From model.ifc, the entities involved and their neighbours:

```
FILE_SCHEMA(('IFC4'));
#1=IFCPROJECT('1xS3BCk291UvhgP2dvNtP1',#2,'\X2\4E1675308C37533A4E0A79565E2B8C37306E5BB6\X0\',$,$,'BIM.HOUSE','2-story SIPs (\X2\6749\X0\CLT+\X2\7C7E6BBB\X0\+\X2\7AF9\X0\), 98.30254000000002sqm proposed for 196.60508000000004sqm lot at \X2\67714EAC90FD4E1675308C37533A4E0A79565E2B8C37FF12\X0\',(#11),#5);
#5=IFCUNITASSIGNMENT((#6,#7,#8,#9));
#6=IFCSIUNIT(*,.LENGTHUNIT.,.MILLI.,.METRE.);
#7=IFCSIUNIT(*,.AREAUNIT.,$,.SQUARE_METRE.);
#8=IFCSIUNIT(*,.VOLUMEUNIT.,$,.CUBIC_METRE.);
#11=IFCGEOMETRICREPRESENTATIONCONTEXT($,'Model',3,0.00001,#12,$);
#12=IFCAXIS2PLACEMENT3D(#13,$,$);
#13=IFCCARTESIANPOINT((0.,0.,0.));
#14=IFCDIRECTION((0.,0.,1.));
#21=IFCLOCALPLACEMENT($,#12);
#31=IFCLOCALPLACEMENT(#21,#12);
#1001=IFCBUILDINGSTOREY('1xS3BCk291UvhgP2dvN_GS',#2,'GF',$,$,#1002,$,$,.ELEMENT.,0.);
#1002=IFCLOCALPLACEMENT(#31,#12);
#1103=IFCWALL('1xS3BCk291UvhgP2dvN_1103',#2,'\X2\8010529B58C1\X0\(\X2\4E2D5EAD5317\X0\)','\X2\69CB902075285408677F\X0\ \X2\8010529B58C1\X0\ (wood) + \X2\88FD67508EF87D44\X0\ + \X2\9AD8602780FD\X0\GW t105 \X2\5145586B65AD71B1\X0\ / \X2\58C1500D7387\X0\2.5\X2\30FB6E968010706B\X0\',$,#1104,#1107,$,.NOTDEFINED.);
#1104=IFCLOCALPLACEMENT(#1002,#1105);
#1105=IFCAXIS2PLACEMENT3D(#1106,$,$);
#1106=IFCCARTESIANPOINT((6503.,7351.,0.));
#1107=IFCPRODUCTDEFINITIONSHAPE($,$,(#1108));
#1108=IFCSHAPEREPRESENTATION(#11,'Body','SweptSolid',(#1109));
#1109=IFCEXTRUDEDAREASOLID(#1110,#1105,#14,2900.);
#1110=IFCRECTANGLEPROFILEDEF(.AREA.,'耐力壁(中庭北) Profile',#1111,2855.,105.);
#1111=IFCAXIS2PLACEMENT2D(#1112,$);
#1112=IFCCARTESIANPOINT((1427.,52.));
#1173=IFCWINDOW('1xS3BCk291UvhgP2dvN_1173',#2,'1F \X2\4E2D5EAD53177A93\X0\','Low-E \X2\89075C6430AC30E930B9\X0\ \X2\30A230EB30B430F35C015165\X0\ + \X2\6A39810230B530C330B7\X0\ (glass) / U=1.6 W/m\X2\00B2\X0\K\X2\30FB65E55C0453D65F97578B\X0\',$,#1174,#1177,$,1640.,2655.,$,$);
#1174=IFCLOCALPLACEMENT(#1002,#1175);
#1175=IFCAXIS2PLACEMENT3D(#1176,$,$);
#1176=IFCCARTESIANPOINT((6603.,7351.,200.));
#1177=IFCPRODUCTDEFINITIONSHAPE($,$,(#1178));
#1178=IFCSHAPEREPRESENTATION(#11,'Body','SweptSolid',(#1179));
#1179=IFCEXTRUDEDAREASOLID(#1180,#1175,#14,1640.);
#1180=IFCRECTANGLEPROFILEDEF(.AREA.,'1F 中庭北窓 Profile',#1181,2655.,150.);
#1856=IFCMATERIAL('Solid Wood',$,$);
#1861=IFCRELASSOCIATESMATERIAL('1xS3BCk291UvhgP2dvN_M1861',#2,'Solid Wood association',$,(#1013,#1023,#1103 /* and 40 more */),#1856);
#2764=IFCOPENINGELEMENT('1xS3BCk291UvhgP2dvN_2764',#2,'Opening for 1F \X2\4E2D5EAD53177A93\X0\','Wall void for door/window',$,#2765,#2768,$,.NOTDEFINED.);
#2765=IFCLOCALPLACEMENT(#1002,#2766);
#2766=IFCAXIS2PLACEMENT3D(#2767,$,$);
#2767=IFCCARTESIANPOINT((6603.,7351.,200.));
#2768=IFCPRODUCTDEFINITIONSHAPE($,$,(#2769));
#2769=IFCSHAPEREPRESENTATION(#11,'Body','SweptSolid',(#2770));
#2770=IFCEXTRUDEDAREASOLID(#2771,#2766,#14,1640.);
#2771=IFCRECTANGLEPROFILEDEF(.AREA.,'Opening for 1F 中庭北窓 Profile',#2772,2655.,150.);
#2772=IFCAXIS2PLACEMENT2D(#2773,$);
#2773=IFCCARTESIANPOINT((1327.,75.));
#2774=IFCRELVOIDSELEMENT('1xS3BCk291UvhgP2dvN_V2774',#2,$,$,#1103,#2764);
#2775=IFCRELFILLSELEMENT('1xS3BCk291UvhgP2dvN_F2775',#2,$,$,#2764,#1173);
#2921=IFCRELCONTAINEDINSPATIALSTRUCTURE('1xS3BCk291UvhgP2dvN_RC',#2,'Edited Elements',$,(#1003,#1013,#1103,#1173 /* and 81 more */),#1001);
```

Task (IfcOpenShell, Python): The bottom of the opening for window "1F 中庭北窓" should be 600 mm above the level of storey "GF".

```python
import numpy as np
import ifcopenshell
import ifcopenshell.api.geometry
import ifcopenshell.geom
import ifcopenshell.util.element
import ifcopenshell.util.placement
import ifcopenshell.util.shape
import ifcopenshell.util.unit

model = ifcopenshell.open("model.ifc")
unit_scale = ifcopenshell.util.unit.calculate_unit_scale(model)

window = model.by_guid("1xS3BCk291UvhgP2dvN_1173")
opening = window.FillsVoids[0].RelatingOpeningElement
storey = ifcopenshell.util.element.get_container(window, ifc_class="IfcBuildingStorey")
level = ifcopenshell.util.placement.get_local_placement(storey.ObjectPlacement)[2, 3]

# The opening's origin need not be at the sill, so measure its lowest point.
shape = ifcopenshell.geom.create_shape(ifcopenshell.geom.settings(), opening)
bottom = ifcopenshell.util.shape.get_shape_bottom_elevation(shape, shape.geometry) / unit_scale
dz = level + 0.6 / unit_scale - bottom

shift = np.array([0.0, 0.0, dz])
# The window is not placed relative to its opening, so move both.
for product in (opening, window):
    matrix = ifcopenshell.util.placement.get_local_placement(product.ObjectPlacement)
    matrix[:3, 3] += shift
    ifcopenshell.api.geometry.edit_object_placement(model, product=product, matrix=matrix, is_si=False)

print(f"moved by {dz * unit_scale:+.3f} m")

model.write("model_v2.ifc")
```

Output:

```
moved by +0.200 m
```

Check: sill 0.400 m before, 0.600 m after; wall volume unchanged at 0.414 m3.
